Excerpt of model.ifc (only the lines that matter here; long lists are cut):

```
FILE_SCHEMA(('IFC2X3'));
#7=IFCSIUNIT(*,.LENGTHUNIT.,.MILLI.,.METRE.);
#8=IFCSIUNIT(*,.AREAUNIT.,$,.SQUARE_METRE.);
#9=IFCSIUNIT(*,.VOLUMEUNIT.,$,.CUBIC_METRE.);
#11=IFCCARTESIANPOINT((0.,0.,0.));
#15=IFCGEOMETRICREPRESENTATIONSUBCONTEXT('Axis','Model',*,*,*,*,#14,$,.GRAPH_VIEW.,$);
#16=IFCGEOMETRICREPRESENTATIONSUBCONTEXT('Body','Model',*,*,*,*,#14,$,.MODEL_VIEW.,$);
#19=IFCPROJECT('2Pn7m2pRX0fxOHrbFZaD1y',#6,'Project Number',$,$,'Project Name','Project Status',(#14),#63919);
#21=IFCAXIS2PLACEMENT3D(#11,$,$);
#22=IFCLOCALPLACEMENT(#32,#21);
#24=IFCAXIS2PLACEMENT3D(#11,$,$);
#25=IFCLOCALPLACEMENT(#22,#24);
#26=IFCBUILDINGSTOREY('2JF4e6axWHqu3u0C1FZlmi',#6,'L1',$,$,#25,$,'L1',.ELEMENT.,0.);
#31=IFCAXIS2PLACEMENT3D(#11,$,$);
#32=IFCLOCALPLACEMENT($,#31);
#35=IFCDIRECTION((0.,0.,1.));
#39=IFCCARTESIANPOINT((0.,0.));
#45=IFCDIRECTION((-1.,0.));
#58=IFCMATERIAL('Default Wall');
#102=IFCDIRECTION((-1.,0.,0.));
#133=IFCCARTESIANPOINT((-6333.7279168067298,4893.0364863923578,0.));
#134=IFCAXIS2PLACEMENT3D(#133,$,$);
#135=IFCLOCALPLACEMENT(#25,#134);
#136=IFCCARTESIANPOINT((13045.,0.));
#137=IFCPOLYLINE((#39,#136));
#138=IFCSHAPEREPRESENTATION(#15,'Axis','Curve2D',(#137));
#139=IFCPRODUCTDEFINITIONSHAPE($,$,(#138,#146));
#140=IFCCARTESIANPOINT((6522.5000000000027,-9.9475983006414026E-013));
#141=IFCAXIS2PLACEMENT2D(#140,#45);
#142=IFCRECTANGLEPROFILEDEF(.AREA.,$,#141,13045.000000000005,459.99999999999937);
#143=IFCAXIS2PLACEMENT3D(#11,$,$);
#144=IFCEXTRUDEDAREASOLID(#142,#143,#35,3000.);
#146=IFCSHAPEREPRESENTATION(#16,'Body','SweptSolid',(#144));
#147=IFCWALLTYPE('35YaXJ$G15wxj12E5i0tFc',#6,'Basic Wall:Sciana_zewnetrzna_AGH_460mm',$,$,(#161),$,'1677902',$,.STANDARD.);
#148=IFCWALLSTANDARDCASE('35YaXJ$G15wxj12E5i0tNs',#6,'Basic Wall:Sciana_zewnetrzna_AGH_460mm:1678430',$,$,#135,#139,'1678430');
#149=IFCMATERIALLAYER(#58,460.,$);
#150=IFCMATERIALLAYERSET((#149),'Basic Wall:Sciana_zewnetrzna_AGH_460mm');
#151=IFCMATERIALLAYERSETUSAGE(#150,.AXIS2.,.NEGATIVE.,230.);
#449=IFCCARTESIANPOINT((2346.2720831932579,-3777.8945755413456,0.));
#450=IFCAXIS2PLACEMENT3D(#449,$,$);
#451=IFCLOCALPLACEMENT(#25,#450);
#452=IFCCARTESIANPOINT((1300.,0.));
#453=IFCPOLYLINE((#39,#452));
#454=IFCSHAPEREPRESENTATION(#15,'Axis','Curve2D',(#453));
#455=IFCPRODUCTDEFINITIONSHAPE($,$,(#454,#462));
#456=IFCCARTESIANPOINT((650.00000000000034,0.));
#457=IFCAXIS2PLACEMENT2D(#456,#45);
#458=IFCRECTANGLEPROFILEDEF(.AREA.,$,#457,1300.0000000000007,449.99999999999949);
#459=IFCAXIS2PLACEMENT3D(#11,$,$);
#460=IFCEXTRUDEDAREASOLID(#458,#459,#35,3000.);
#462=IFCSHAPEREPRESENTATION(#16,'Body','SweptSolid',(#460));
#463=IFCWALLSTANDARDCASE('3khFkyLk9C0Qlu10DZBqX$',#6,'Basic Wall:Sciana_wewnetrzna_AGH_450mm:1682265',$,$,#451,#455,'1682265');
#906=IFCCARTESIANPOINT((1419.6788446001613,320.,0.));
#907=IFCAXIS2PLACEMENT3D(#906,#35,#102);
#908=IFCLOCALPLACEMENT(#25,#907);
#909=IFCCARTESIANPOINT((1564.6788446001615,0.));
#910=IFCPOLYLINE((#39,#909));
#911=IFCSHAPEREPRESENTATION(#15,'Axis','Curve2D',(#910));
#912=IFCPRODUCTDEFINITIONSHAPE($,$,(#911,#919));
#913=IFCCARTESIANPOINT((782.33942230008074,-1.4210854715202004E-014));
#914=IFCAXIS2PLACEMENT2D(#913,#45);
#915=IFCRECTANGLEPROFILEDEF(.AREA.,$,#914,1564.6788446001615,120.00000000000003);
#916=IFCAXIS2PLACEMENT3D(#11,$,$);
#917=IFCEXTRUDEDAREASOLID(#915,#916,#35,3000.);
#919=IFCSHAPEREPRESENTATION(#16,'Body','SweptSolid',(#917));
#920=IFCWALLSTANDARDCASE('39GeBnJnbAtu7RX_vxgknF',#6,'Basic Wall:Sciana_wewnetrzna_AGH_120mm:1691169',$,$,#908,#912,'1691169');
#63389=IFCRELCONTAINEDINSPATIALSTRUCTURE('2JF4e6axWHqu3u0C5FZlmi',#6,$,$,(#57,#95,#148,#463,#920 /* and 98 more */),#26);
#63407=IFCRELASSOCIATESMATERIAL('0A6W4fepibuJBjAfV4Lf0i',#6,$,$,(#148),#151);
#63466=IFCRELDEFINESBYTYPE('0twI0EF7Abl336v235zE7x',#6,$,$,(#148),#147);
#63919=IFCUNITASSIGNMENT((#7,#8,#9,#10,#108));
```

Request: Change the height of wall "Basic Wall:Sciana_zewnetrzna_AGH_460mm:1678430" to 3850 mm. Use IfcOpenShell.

```python
import ifcopenshell
import ifcopenshell.geom
import ifcopenshell.util.representation
import ifcopenshell.util.shape
import ifcopenshell.util.unit

model = ifcopenshell.open("model.ifc")
unit_scale = ifcopenshell.util.unit.calculate_unit_scale(model)
settings = ifcopenshell.geom.settings()


def volume(element):
    """Net volume in cubic metres, openings subtracted."""
    shape = ifcopenshell.geom.create_shape(settings, element)
    return ifcopenshell.util.shape.get_volume(shape.geometry)


wall = model.by_guid("35YaXJ$G15wxj12E5i0tNs")
before = volume(wall)

body = ifcopenshell.util.representation.get_representation(wall, "Model", "Body")
solid = body.Items[0]
old_height = solid.Depth
solid.Depth = 3.85 / unit_scale
after = volume(wall)

print(f"height {old_height:g} -> {solid.Depth:g}, volume {before:.3f} -> {after:.3f} m3")

model.write("model-out.ifc")
```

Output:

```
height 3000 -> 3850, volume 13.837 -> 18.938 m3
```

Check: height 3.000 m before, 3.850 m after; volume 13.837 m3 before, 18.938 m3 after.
